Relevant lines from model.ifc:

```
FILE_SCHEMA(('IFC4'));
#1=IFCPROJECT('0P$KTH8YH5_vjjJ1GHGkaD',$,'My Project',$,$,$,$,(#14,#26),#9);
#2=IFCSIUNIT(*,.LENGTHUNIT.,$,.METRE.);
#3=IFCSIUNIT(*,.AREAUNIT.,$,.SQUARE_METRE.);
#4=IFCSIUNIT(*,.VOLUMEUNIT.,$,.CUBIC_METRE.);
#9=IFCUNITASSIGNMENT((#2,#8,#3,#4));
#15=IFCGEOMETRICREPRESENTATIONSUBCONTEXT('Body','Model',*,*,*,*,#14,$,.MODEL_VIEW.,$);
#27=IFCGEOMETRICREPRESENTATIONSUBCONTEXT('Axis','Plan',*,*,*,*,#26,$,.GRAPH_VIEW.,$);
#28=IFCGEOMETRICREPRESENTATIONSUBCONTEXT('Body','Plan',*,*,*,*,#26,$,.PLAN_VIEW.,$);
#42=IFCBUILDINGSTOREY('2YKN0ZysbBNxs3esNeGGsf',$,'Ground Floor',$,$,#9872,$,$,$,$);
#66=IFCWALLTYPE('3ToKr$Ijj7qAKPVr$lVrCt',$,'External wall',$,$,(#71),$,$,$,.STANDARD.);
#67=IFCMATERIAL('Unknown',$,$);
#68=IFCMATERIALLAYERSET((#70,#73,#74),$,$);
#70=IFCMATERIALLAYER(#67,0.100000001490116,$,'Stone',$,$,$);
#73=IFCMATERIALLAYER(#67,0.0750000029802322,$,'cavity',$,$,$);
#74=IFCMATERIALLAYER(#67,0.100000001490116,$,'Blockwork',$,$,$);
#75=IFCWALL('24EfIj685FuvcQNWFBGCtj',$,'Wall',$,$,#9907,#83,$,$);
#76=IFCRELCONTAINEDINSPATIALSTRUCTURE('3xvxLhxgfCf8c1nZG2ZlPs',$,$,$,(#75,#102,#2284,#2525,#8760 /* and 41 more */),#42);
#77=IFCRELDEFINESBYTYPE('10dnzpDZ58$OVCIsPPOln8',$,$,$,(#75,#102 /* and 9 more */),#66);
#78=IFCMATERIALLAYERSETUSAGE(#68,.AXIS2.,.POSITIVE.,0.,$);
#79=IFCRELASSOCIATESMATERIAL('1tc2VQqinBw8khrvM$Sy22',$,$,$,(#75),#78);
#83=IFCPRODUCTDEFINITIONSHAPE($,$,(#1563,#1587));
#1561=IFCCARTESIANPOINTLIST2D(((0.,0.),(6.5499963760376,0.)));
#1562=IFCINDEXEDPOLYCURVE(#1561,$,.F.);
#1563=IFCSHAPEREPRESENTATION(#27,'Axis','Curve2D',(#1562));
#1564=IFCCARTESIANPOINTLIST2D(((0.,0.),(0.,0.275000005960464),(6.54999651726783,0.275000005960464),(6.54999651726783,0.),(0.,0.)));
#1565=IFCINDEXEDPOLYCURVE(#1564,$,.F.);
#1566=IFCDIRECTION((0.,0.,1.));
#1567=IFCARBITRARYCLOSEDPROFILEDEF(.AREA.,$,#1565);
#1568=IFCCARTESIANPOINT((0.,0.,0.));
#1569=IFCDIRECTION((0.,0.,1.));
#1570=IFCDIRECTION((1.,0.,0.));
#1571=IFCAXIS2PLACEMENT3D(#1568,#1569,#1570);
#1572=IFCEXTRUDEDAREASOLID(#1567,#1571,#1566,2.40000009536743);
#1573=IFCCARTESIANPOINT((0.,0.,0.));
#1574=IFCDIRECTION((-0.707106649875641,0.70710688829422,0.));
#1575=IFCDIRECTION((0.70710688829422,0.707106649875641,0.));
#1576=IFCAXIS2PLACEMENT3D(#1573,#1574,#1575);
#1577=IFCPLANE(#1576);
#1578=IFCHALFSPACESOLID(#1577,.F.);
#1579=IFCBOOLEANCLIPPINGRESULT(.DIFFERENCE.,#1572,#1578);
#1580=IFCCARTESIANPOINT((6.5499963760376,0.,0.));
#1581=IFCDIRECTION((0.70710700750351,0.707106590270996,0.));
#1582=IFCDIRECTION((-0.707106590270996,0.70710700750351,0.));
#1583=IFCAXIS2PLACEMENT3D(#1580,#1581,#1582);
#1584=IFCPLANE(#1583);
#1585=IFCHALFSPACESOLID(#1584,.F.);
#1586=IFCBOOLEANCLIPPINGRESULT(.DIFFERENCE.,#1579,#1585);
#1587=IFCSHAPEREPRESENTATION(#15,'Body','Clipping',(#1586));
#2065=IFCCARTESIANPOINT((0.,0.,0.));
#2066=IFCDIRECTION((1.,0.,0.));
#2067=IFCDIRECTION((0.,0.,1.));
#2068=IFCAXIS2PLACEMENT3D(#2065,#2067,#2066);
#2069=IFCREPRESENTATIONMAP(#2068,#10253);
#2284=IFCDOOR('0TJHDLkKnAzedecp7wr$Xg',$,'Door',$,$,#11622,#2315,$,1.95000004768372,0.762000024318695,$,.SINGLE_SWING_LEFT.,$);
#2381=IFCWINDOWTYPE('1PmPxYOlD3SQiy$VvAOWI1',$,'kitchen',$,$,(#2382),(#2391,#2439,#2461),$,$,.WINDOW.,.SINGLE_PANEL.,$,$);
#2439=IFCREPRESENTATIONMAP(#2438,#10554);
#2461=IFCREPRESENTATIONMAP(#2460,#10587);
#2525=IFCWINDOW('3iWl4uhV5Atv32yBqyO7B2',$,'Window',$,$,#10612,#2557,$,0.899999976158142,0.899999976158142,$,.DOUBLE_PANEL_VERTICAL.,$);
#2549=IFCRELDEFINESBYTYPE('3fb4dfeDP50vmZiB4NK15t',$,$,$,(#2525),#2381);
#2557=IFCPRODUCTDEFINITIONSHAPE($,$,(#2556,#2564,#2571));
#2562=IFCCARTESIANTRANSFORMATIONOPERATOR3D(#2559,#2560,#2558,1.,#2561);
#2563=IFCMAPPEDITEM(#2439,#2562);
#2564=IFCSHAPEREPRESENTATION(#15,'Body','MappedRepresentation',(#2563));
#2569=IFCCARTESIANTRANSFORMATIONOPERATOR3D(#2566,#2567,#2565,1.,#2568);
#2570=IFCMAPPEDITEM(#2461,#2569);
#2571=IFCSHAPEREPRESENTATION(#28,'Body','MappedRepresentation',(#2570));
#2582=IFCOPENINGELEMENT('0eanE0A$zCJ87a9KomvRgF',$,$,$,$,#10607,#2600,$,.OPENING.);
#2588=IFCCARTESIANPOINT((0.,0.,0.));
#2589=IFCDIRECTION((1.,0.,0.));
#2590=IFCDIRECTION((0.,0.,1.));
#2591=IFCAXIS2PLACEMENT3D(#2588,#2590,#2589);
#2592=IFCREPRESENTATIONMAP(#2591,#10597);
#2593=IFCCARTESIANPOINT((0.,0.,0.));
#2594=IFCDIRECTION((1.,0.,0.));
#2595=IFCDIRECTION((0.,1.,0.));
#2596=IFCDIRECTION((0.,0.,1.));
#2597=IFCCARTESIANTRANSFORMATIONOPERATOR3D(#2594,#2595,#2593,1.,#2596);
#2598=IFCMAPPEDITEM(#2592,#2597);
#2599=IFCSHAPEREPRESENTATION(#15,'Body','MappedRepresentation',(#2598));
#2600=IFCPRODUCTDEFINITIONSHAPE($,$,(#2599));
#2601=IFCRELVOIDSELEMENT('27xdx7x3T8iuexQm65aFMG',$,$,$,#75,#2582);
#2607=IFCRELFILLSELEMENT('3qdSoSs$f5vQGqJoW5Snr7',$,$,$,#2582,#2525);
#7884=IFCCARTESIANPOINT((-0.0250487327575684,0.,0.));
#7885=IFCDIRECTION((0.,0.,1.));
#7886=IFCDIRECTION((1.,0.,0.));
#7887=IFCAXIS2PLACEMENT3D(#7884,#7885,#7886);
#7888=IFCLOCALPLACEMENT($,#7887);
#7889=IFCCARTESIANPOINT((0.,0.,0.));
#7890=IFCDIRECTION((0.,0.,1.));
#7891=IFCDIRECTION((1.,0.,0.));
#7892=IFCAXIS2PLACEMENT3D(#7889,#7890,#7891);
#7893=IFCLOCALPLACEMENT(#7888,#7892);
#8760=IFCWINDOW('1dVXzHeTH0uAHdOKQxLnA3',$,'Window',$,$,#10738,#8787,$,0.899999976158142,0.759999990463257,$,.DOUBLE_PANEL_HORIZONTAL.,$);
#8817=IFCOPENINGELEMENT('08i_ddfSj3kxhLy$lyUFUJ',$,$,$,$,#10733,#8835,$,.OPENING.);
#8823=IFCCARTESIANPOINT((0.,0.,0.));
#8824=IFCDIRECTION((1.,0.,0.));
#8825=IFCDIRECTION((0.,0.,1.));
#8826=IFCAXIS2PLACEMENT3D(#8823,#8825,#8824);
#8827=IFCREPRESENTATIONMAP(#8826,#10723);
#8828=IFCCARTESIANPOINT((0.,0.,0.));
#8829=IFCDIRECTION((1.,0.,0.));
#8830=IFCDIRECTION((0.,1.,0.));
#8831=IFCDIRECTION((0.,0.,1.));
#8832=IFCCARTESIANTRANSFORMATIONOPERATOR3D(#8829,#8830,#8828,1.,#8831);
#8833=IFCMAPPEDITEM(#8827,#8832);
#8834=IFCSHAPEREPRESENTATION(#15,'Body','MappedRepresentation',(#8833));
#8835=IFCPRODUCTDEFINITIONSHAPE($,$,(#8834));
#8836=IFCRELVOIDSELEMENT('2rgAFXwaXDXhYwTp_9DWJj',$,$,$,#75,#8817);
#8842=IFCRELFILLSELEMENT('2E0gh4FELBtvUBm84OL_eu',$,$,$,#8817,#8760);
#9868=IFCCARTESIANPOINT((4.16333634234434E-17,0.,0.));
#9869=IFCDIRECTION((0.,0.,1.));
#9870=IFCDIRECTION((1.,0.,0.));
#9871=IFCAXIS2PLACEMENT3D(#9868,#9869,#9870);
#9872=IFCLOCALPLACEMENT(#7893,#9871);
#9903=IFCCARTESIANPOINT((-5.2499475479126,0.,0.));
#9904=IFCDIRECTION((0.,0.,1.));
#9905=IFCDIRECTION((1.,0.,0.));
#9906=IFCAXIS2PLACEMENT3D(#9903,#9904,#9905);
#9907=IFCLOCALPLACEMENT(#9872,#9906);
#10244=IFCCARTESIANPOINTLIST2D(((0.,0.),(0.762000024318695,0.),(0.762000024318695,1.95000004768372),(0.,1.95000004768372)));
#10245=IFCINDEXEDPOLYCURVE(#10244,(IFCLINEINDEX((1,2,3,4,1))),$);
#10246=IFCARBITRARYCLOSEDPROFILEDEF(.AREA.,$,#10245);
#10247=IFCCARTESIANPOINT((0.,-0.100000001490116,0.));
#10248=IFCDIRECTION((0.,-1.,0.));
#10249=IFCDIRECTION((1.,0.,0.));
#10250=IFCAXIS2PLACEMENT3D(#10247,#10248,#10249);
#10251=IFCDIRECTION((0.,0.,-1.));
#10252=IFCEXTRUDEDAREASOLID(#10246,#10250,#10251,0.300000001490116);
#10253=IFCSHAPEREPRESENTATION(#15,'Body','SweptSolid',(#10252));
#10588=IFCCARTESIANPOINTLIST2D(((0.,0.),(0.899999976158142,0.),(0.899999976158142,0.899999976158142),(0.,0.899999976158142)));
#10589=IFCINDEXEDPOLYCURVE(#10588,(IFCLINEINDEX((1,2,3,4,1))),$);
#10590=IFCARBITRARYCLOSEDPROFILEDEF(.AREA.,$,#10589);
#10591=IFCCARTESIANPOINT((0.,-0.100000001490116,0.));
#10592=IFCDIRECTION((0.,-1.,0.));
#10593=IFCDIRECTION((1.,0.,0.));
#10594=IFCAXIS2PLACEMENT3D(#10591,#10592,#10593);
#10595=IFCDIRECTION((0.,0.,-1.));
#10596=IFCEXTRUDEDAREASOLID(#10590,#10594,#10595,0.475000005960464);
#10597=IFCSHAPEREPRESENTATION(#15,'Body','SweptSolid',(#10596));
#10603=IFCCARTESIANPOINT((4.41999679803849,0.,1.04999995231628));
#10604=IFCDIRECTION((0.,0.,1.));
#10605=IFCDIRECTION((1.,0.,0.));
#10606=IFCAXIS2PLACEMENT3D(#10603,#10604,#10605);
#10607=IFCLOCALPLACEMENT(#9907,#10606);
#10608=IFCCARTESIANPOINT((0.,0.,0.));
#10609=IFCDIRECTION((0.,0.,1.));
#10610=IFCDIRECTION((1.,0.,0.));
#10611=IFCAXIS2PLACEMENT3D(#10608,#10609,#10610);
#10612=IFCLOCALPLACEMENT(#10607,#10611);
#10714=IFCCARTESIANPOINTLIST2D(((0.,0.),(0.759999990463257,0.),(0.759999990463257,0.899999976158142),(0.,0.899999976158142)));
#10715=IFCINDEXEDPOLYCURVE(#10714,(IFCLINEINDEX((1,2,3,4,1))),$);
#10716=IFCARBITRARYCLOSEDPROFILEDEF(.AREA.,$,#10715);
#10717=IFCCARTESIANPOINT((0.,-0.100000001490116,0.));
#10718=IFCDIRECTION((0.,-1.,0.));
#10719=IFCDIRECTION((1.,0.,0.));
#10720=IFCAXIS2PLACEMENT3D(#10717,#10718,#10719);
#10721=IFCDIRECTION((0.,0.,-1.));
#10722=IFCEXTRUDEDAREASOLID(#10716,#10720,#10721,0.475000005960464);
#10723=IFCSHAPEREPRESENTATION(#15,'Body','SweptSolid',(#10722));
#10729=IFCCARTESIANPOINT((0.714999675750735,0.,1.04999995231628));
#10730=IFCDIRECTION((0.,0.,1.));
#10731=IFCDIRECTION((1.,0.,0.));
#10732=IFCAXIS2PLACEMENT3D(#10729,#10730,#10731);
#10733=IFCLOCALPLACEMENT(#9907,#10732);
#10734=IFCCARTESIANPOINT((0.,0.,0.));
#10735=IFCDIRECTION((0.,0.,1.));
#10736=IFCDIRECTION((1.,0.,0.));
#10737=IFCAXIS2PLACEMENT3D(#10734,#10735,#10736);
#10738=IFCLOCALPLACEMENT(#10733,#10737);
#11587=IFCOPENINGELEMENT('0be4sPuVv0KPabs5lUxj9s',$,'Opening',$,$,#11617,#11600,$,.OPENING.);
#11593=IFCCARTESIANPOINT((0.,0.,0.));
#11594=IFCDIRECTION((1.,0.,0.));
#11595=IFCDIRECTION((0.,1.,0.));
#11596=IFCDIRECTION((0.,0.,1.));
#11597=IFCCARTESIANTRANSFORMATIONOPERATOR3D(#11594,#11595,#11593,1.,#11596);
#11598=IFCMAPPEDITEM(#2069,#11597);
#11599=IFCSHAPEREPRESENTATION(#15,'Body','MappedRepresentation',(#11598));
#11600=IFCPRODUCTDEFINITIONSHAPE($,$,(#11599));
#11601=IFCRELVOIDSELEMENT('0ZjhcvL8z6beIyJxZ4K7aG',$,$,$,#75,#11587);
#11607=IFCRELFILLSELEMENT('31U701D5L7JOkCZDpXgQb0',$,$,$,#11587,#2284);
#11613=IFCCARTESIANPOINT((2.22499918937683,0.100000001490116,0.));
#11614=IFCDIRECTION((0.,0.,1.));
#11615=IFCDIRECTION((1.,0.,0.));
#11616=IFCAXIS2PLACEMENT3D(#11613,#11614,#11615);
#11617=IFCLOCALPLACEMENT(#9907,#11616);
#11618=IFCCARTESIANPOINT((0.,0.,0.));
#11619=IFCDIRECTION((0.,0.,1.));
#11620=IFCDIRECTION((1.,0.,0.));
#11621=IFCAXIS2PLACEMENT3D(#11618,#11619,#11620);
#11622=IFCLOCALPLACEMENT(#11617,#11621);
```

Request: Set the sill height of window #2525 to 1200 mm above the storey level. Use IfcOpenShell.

```python
import numpy as np
import ifcopenshell
import ifcopenshell.api.geometry
import ifcopenshell.geom
import ifcopenshell.util.element
import ifcopenshell.util.placement
import ifcopenshell.util.shape
import ifcopenshell.util.unit

model = ifcopenshell.open("model.ifc")
unit_scale = ifcopenshell.util.unit.calculate_unit_scale(model)

window = model.by_guid("3iWl4uhV5Atv32yBqyO7B2")
opening = window.FillsVoids[0].RelatingOpeningElement
storey = ifcopenshell.util.element.get_container(window, ifc_class="IfcBuildingStorey")
level = ifcopenshell.util.placement.get_local_placement(storey.ObjectPlacement)[2, 3]

# The opening's origin need not be at the sill, so measure its lowest point.
shape = ifcopenshell.geom.create_shape(ifcopenshell.geom.settings(), opening)
bottom = ifcopenshell.util.shape.get_shape_bottom_elevation(shape, shape.geometry) / unit_scale
dz = level + 1.2 / unit_scale - bottom

shift = np.array([0.0, 0.0, dz])
# The window is placed relative to its opening, so it follows when the opening moves.
matrix = ifcopenshell.util.placement.get_local_placement(opening.ObjectPlacement)
matrix[:3, 3] += shift
ifcopenshell.api.geometry.edit_object_placement(
    model, product=opening, matrix=matrix, is_si=False, should_transform_children=True
)

print(f"moved by {dz * unit_scale:+.3f} m")

model.write("model_rev.ifc")
```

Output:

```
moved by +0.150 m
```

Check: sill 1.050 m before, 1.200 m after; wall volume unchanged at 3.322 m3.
